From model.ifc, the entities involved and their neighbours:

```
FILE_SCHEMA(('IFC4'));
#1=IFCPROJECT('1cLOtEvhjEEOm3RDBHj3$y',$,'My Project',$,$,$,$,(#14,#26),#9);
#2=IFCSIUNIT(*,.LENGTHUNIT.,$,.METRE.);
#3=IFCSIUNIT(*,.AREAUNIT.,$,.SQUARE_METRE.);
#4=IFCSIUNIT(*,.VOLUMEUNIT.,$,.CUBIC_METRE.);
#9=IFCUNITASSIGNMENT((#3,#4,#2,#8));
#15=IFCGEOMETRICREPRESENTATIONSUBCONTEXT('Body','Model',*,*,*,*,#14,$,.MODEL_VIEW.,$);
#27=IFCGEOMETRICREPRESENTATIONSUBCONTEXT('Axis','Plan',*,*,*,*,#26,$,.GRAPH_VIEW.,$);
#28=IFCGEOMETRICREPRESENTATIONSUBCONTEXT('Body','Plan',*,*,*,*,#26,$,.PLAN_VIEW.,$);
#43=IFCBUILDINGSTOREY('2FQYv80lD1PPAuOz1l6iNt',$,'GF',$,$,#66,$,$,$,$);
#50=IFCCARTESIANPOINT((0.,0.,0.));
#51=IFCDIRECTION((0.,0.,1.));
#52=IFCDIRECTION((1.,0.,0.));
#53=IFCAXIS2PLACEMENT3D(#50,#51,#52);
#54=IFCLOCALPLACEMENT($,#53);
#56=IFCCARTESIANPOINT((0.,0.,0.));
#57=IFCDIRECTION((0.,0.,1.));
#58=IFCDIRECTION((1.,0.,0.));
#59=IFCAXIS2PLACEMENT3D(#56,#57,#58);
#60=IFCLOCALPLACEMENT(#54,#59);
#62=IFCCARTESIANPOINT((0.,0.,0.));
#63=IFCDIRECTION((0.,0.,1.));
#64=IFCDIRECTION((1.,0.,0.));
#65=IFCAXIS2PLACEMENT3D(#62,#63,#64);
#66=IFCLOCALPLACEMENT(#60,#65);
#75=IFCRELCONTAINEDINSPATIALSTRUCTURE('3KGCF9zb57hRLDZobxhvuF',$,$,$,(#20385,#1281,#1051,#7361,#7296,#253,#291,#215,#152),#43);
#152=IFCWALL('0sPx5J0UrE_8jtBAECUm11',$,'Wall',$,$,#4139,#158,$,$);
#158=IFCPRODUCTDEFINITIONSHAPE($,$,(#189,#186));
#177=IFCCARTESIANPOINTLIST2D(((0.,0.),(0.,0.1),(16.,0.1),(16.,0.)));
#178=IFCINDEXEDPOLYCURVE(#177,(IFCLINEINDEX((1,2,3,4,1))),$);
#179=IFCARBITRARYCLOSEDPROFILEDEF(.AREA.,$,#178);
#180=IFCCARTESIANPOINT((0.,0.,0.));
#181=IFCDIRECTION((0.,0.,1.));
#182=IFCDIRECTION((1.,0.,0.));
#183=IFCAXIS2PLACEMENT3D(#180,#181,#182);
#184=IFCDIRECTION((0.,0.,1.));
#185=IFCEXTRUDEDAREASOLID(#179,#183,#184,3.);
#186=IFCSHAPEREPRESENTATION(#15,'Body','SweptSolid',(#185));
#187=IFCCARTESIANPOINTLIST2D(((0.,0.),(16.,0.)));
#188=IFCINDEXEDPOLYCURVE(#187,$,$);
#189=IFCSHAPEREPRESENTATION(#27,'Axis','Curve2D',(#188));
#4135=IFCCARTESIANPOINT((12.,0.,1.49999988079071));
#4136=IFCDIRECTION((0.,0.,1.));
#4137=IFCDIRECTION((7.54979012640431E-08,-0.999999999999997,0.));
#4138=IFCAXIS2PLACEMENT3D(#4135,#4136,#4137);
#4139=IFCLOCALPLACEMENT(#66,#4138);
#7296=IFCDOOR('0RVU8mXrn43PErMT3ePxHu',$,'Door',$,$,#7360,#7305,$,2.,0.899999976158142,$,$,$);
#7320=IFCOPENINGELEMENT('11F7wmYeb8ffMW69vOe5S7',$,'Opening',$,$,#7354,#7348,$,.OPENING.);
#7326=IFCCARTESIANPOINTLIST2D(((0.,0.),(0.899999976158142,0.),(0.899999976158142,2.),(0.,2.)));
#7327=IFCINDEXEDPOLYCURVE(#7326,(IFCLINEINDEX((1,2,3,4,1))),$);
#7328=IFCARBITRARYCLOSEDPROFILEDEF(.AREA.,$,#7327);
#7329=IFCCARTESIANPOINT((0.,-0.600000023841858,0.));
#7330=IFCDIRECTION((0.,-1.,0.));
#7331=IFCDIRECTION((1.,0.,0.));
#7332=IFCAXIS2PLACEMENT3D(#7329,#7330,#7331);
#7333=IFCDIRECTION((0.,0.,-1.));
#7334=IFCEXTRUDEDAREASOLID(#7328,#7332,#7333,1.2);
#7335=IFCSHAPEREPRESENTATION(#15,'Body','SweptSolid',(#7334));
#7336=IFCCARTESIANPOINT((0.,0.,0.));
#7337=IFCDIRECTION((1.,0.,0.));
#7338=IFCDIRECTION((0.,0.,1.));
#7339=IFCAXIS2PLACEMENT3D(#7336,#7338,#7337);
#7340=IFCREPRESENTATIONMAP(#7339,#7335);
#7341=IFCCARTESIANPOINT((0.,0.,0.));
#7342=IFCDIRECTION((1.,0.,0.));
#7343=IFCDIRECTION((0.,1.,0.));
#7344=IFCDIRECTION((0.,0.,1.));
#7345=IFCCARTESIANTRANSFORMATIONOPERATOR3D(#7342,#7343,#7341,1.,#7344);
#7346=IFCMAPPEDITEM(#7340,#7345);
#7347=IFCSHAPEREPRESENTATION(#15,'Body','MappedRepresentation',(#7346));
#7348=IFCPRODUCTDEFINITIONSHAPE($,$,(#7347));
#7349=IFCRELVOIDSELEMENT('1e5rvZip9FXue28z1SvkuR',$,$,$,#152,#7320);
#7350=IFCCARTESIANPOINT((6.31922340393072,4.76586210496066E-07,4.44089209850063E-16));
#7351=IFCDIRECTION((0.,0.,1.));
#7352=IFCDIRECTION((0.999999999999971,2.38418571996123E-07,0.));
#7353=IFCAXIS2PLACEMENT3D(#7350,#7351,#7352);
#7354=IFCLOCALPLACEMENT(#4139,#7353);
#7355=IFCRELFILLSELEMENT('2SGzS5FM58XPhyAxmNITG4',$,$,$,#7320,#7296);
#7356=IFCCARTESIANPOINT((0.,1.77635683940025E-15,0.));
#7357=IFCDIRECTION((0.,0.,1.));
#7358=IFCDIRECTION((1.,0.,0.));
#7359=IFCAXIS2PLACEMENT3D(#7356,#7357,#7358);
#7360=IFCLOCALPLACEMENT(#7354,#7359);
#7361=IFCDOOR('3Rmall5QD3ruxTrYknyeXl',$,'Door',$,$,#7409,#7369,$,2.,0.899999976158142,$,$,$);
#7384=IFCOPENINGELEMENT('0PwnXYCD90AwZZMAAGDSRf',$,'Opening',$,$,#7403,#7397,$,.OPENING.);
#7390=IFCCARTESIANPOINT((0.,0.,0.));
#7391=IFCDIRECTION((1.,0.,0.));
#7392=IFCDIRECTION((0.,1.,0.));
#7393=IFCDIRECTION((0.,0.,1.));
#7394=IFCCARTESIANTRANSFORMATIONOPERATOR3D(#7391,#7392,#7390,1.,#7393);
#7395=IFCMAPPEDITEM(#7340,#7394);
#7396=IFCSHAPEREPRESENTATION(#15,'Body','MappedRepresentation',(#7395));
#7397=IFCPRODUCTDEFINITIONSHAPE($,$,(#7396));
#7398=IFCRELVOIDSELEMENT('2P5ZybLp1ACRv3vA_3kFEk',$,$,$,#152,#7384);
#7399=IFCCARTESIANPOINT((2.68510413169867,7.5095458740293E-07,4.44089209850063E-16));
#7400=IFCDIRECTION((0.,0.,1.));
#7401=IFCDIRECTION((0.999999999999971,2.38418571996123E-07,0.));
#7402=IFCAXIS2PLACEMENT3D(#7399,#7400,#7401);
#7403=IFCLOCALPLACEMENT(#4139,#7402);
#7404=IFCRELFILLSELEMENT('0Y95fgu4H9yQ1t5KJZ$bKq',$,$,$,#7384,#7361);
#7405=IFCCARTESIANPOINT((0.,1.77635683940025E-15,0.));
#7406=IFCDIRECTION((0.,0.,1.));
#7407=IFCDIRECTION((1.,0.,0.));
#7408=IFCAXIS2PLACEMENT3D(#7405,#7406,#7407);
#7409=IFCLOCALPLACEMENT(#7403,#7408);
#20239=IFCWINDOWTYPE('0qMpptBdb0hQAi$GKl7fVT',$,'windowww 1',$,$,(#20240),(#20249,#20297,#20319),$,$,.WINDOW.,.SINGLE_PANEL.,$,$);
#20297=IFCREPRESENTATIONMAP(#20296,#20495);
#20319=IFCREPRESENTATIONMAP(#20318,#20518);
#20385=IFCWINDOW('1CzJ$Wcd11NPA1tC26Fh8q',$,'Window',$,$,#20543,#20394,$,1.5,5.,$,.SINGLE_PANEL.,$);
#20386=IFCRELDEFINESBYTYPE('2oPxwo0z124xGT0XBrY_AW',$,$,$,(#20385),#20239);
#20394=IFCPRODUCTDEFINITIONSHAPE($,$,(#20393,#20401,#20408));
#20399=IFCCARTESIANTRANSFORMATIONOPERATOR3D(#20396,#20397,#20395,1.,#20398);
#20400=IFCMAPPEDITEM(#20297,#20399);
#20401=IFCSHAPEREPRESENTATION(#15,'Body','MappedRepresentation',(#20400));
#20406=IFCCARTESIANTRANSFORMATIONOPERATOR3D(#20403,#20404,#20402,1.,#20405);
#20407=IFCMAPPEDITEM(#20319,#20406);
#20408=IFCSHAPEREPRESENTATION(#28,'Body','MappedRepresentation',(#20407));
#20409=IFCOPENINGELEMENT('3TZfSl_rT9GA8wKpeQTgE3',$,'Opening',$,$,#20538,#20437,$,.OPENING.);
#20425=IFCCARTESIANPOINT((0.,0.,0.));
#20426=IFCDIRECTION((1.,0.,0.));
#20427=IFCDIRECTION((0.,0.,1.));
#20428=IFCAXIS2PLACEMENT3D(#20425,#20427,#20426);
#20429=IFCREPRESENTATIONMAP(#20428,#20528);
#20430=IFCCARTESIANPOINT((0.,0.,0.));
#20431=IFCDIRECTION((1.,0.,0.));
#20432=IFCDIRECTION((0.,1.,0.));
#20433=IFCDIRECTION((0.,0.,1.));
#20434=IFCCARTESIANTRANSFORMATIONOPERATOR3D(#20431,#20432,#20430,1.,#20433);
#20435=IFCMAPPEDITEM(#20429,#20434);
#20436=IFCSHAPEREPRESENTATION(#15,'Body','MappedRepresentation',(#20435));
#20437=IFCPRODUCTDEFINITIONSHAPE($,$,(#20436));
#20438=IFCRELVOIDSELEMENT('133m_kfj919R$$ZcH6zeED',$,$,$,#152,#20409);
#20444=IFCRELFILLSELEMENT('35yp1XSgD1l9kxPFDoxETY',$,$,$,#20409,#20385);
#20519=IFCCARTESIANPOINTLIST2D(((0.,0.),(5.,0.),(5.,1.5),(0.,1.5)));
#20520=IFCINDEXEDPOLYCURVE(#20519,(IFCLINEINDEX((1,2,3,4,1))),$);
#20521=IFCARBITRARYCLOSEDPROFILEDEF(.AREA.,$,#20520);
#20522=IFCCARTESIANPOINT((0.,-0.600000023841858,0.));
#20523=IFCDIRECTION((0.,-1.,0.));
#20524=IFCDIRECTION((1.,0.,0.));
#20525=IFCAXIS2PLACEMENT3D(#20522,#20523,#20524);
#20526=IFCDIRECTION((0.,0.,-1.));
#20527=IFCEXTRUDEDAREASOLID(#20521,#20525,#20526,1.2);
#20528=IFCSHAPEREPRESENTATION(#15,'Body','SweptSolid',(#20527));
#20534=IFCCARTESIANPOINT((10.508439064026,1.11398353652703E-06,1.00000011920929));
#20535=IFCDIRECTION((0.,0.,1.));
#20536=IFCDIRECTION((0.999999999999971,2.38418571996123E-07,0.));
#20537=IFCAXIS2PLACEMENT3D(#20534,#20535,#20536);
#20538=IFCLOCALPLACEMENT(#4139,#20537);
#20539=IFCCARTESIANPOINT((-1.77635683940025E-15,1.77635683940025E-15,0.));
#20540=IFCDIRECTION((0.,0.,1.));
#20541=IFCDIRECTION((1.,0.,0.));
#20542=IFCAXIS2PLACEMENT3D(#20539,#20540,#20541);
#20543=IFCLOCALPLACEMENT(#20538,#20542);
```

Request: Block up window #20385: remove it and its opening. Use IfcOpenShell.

```python
import ifcopenshell
import ifcopenshell.api.feature
import ifcopenshell.api.root
import ifcopenshell.geom
import ifcopenshell.util.shape

model = ifcopenshell.open("model.ifc")
settings = ifcopenshell.geom.settings()


def volume(element):
    """Net volume in cubic metres, openings subtracted."""
    shape = ifcopenshell.geom.create_shape(settings, element)
    return ifcopenshell.util.shape.get_volume(shape.geometry)


window = model.by_id(20385)
opening = window.FillsVoids[0].RelatingOpeningElement
wall = opening.VoidsElements[0].RelatingBuildingElement
before = volume(wall)

ifcopenshell.api.root.remove_product(model, product=window)
ifcopenshell.api.feature.remove_feature(model, feature=opening)

after = volume(wall)

print(f"wall volume {before:.3f} -> {after:.3f} m3")

model.write("model_v2.ifc")
```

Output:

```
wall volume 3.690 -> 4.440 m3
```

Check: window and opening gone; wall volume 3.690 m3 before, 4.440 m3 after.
